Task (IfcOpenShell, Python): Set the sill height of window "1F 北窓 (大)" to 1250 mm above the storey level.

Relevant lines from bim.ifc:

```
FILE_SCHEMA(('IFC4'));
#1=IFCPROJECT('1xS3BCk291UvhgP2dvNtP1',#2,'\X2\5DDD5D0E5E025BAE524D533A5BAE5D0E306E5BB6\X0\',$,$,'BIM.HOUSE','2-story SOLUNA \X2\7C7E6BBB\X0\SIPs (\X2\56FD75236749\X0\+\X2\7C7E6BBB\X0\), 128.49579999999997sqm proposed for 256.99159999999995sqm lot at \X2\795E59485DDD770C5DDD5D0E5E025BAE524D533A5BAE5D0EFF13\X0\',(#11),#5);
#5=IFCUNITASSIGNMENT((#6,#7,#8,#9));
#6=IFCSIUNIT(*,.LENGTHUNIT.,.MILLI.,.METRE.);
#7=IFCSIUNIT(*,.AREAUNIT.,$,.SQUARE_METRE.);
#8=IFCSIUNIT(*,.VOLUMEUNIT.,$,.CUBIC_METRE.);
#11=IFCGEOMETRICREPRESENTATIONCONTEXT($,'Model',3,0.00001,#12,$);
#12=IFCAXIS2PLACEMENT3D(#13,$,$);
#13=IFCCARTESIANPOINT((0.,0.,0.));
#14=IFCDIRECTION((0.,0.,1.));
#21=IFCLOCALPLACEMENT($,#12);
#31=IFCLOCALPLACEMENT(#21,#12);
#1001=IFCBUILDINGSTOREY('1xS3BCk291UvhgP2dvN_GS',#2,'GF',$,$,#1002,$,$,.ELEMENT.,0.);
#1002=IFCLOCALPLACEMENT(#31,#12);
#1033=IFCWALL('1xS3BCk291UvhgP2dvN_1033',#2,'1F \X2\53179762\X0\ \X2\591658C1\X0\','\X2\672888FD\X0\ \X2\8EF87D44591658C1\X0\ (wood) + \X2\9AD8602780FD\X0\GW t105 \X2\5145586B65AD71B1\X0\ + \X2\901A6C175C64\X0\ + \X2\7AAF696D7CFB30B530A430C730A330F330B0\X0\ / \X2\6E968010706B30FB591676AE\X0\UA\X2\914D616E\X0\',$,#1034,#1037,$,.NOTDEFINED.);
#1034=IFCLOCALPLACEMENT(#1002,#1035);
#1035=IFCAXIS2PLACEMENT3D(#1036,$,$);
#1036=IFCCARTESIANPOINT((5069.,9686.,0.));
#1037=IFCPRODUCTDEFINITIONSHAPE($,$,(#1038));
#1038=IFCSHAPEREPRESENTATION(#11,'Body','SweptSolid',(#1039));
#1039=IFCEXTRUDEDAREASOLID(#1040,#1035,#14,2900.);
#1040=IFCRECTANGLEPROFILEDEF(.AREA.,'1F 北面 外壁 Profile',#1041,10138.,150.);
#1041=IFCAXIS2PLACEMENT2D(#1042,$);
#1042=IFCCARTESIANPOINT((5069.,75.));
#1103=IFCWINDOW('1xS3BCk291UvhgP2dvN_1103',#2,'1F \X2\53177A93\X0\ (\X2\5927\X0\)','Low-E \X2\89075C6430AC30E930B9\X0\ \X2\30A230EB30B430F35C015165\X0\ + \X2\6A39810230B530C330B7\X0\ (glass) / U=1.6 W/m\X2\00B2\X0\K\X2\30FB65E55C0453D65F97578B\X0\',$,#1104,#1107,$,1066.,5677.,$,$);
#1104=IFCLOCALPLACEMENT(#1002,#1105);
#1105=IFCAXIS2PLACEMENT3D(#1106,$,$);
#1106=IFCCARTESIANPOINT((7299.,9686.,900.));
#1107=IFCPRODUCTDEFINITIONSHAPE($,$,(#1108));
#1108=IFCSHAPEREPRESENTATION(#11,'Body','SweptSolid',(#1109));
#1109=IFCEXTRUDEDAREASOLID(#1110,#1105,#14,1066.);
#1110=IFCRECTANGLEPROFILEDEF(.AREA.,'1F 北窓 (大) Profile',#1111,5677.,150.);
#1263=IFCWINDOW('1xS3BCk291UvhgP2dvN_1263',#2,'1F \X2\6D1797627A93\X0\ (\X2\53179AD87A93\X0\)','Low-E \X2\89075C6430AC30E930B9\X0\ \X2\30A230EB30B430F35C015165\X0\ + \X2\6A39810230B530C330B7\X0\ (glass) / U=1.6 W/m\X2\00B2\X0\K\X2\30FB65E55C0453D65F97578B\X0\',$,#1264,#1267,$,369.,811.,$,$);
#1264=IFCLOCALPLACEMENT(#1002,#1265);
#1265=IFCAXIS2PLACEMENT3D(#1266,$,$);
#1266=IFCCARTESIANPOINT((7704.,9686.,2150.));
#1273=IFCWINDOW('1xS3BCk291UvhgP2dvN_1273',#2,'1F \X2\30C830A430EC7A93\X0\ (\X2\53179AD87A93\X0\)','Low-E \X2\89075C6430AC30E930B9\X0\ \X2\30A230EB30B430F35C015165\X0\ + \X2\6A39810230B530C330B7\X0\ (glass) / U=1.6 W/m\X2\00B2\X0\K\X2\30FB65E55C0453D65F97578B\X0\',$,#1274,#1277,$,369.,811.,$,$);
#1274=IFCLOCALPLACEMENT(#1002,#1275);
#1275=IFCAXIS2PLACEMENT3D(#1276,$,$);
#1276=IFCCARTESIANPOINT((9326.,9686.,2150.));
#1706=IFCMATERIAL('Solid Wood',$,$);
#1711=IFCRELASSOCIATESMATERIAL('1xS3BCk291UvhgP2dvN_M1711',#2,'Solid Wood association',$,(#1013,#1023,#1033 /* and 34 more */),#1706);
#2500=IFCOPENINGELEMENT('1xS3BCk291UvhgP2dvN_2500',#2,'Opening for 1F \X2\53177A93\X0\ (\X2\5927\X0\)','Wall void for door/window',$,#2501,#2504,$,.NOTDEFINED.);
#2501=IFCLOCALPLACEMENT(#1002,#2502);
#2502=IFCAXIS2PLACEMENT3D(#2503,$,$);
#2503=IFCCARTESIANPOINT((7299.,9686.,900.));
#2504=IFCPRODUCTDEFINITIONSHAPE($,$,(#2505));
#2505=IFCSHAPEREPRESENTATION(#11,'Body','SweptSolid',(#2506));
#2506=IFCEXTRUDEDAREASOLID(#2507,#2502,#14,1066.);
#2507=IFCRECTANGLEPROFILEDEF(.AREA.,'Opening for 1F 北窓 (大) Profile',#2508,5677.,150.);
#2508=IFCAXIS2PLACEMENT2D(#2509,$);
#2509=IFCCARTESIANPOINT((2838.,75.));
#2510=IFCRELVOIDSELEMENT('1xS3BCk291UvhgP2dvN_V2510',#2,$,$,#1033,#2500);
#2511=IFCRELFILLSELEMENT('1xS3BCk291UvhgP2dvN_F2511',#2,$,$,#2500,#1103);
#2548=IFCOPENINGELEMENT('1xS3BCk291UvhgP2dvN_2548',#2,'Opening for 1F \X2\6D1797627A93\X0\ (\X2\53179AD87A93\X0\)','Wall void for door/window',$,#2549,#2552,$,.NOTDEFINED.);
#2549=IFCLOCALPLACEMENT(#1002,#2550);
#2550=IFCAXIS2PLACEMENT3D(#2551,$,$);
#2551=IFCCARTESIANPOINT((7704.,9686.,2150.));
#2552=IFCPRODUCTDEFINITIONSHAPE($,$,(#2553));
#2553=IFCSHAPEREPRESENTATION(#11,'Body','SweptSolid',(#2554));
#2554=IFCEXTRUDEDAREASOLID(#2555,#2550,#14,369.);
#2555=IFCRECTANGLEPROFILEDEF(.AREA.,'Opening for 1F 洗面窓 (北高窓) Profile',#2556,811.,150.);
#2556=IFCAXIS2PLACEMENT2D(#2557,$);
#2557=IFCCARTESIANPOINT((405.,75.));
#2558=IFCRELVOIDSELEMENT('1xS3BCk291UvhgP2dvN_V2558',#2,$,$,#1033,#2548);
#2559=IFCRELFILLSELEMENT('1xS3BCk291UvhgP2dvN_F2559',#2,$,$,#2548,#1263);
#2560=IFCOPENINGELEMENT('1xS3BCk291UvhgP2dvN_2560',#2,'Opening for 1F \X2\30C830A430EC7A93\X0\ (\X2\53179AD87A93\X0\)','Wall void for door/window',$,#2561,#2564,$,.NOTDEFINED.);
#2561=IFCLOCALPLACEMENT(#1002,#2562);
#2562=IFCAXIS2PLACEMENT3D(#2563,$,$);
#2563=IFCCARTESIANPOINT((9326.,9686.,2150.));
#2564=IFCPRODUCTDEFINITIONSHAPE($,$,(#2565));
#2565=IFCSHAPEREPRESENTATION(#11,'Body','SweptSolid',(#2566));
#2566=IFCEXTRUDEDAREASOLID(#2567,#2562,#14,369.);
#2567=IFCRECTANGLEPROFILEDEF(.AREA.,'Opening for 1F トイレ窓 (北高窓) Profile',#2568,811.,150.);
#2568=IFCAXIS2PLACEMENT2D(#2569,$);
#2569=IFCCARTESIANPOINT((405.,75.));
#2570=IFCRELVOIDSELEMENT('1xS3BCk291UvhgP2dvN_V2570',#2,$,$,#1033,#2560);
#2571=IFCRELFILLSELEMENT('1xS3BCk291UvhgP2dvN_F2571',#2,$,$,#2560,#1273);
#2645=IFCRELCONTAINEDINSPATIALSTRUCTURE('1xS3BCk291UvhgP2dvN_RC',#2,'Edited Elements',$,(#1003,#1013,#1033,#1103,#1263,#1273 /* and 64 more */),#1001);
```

```python
import numpy as np
import ifcopenshell
import ifcopenshell.api.geometry
import ifcopenshell.geom
import ifcopenshell.util.element
import ifcopenshell.util.placement
import ifcopenshell.util.shape
import ifcopenshell.util.unit

model = ifcopenshell.open("bim.ifc")
unit_scale = ifcopenshell.util.unit.calculate_unit_scale(model)

window = model.by_guid("1xS3BCk291UvhgP2dvN_1103")
opening = window.FillsVoids[0].RelatingOpeningElement
storey = ifcopenshell.util.element.get_container(window, ifc_class="IfcBuildingStorey")
level = ifcopenshell.util.placement.get_local_placement(storey.ObjectPlacement)[2, 3]

# The opening's origin need not be at the sill, so measure its lowest point.
shape = ifcopenshell.geom.create_shape(ifcopenshell.geom.settings(), opening)
bottom = ifcopenshell.util.shape.get_shape_bottom_elevation(shape, shape.geometry) / unit_scale
dz = level + 1.25 / unit_scale - bottom

shift = np.array([0.0, 0.0, dz])
# The window is not placed relative to its opening, so move both.
for product in (opening, window):
    matrix = ifcopenshell.util.placement.get_local_placement(product.ObjectPlacement)
    matrix[:3, 3] += shift
    ifcopenshell.api.geometry.edit_object_placement(model, product=product, matrix=matrix, is_si=False)

print(f"moved by {dz * unit_scale:+.3f} m")

model.write("bim_edited.ifc")
```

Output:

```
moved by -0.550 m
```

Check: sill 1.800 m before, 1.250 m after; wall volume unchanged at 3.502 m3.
